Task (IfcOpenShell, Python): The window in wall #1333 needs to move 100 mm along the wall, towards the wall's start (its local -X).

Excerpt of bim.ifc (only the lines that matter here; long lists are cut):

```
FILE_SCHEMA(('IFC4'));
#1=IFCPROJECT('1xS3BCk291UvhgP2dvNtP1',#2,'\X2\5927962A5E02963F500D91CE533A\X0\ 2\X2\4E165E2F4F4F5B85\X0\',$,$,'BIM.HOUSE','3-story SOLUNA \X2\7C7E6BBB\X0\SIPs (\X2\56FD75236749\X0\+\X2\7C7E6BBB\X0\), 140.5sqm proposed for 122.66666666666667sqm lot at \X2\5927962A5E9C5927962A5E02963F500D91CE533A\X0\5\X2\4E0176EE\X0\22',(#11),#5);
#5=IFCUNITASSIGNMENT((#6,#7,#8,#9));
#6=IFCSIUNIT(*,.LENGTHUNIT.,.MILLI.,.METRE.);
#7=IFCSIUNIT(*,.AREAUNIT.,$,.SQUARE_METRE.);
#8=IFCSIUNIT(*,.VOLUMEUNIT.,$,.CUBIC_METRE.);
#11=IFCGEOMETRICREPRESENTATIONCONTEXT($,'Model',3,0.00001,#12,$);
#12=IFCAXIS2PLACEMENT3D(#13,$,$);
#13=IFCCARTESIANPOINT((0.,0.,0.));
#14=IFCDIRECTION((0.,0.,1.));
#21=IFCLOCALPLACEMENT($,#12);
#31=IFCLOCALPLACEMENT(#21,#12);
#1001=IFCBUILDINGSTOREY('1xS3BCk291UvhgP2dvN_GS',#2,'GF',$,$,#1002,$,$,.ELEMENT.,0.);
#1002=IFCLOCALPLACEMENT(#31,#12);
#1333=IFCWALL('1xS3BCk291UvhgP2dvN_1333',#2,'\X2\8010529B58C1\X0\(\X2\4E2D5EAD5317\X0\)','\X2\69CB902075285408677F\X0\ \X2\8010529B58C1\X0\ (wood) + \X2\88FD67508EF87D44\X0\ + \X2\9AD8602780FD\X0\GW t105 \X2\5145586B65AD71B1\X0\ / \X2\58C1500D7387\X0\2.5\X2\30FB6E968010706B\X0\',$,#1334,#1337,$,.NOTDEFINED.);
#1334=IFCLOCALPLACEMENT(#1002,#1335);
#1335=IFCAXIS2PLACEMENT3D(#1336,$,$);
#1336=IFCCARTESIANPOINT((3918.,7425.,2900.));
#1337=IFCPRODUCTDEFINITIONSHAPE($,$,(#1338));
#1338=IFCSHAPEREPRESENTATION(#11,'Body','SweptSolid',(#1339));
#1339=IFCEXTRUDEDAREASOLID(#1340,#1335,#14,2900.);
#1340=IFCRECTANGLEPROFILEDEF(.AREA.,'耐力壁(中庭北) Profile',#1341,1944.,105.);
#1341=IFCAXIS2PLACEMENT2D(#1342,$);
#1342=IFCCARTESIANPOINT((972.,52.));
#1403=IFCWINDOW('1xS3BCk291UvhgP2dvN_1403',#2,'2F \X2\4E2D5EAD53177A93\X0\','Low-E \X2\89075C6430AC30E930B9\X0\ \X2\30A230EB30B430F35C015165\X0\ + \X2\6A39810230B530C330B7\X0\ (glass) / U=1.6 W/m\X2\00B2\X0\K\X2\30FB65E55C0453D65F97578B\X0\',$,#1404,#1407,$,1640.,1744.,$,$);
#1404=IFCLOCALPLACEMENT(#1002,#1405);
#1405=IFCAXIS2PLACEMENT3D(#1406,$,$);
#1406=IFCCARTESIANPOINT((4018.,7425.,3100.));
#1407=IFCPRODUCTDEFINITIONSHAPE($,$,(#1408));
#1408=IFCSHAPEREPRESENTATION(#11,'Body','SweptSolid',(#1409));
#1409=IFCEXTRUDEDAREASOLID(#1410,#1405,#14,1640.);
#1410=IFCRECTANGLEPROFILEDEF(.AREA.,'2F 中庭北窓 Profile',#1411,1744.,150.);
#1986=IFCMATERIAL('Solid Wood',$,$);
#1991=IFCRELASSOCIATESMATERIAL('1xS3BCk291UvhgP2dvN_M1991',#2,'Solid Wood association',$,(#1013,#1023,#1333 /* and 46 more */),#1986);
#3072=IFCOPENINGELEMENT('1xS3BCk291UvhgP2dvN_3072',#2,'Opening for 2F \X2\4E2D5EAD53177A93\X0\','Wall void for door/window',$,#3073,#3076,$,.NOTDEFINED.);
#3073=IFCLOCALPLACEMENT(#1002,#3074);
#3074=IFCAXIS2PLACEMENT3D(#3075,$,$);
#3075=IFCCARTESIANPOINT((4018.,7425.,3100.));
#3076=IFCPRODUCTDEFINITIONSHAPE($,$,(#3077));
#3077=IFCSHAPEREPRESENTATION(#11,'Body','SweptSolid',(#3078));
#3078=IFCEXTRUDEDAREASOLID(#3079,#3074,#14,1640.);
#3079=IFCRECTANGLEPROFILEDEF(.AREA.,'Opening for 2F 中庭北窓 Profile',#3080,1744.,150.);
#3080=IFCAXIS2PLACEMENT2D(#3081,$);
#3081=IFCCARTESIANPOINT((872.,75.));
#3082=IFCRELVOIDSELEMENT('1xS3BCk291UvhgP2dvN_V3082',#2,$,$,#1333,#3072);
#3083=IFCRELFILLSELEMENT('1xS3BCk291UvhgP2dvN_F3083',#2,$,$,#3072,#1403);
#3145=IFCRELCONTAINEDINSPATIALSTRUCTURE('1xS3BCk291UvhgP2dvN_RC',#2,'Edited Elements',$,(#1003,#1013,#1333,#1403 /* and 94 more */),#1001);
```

```python
import ifcopenshell
import ifcopenshell.api.geometry
import ifcopenshell.util.placement
import ifcopenshell.util.unit

model = ifcopenshell.open("bim.ifc")
unit_scale = ifcopenshell.util.unit.calculate_unit_scale(model)

window = model.by_guid("1xS3BCk291UvhgP2dvN_1403")
opening = window.FillsVoids[0].RelatingOpeningElement
wall = opening.VoidsElements[0].RelatingBuildingElement

wall_matrix = ifcopenshell.util.placement.get_local_placement(wall.ObjectPlacement)
shift = wall_matrix[:3, 0] * -0.1 / unit_scale
before = ifcopenshell.util.placement.get_local_placement(window.ObjectPlacement)[:3, 3].copy()

# The window is not placed relative to its opening, so move both.
for product in (opening, window):
    matrix = ifcopenshell.util.placement.get_local_placement(product.ObjectPlacement)
    matrix[:3, 3] += shift
    ifcopenshell.api.geometry.edit_object_placement(model, product=product, matrix=matrix, is_si=False)

after = ifcopenshell.util.placement.get_local_placement(window.ObjectPlacement)[:3, 3]
print("window moved by", (after - before).round(3) + 0.0)

model.write("bim_edited.ifc")
```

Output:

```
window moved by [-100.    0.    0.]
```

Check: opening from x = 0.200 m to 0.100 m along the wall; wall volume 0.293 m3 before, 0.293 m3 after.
